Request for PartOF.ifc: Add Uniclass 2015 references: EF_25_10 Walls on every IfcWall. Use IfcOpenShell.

First a look at what the model holds.

```python
import ifcopenshell

model = ifcopenshell.open("PartOF.ifc")
print(model.schema)
print("classifications:", [c.Name for c in model.by_type("IfcClassification")])
for ifc_class in ("IfcDoor", "IfcRoof", "IfcStair", "IfcWall", "IfcWindow"):
    print(ifc_class, len(model.by_type(ifc_class)))
```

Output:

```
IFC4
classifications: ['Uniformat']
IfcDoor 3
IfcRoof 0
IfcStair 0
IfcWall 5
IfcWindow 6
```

```python
import ifcopenshell
import ifcopenshell.api.classification

model = ifcopenshell.open("PartOF.ifc")

system = ifcopenshell.api.classification.add_classification(model, classification="Uniclass 2015")

codes = {
    "IfcWall": ("EF_25_10", "Walls"),
}
for ifc_class, (code, name) in codes.items():
    products = model.by_type(ifc_class)
    ifcopenshell.api.classification.add_reference(
        model, products=products, classification=system, identification=code, name=name
    )
    print(code, len(products))

model.write("PartOF_rev.ifc")
```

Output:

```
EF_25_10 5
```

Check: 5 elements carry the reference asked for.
